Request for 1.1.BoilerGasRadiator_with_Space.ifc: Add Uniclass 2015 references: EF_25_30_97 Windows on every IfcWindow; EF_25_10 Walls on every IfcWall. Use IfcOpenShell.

First a look at what the model holds.

```python
import ifcopenshell

model = ifcopenshell.open("1.1.BoilerGasRadiator_with_Space.ifc")
print(model.schema)
print("classifications:", [c.Name for c in model.by_type("IfcClassification")])
for ifc_class in ("IfcDoor", "IfcRoof", "IfcStair", "IfcWall", "IfcWindow"):
    print(ifc_class, len(model.by_type(ifc_class)))
```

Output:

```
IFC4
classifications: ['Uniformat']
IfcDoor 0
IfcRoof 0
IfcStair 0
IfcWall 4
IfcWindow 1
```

```python
import ifcopenshell
import ifcopenshell.api.classification

model = ifcopenshell.open("1.1.BoilerGasRadiator_with_Space.ifc")

system = ifcopenshell.api.classification.add_classification(model, classification="Uniclass 2015")

codes = {
    "IfcWindow": ("EF_25_30_97", "Windows"),
    "IfcWall": ("EF_25_10", "Walls"),
}
for ifc_class, (code, name) in codes.items():
    products = model.by_type(ifc_class)
    ifcopenshell.api.classification.add_reference(
        model, products=products, classification=system, identification=code, name=name
    )
    print(code, len(products))

model.write("1.1.BoilerGasRadiator_with_Space_rev.ifc")
```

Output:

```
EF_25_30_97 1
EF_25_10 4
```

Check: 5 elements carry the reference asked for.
